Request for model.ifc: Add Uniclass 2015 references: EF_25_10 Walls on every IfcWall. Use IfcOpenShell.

First a look at what the model holds.

```python
import ifcopenshell

model = ifcopenshell.open("model.ifc")
print(model.schema)
print("classifications:", [c.Name for c in model.by_type("IfcClassification")])
for ifc_class in ("IfcDoor", "IfcRoof", "IfcStair", "IfcWall", "IfcWindow"):
    print(ifc_class, len(model.by_type(ifc_class)))
```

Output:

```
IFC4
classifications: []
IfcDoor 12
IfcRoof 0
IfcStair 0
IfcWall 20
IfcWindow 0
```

```python
import ifcopenshell
import ifcopenshell.api.classification

model = ifcopenshell.open("model.ifc")

system = ifcopenshell.api.classification.add_classification(model, classification="Uniclass 2015")

codes = {
    "IfcWall": ("EF_25_10", "Walls"),
}
for ifc_class, (code, name) in codes.items():
    products = model.by_type(ifc_class)
    ifcopenshell.api.classification.add_reference(
        model, products=products, classification=system, identification=code, name=name
    )
    print(code, len(products))

model.write("model_edited.ifc")
```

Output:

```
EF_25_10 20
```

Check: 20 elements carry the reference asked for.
